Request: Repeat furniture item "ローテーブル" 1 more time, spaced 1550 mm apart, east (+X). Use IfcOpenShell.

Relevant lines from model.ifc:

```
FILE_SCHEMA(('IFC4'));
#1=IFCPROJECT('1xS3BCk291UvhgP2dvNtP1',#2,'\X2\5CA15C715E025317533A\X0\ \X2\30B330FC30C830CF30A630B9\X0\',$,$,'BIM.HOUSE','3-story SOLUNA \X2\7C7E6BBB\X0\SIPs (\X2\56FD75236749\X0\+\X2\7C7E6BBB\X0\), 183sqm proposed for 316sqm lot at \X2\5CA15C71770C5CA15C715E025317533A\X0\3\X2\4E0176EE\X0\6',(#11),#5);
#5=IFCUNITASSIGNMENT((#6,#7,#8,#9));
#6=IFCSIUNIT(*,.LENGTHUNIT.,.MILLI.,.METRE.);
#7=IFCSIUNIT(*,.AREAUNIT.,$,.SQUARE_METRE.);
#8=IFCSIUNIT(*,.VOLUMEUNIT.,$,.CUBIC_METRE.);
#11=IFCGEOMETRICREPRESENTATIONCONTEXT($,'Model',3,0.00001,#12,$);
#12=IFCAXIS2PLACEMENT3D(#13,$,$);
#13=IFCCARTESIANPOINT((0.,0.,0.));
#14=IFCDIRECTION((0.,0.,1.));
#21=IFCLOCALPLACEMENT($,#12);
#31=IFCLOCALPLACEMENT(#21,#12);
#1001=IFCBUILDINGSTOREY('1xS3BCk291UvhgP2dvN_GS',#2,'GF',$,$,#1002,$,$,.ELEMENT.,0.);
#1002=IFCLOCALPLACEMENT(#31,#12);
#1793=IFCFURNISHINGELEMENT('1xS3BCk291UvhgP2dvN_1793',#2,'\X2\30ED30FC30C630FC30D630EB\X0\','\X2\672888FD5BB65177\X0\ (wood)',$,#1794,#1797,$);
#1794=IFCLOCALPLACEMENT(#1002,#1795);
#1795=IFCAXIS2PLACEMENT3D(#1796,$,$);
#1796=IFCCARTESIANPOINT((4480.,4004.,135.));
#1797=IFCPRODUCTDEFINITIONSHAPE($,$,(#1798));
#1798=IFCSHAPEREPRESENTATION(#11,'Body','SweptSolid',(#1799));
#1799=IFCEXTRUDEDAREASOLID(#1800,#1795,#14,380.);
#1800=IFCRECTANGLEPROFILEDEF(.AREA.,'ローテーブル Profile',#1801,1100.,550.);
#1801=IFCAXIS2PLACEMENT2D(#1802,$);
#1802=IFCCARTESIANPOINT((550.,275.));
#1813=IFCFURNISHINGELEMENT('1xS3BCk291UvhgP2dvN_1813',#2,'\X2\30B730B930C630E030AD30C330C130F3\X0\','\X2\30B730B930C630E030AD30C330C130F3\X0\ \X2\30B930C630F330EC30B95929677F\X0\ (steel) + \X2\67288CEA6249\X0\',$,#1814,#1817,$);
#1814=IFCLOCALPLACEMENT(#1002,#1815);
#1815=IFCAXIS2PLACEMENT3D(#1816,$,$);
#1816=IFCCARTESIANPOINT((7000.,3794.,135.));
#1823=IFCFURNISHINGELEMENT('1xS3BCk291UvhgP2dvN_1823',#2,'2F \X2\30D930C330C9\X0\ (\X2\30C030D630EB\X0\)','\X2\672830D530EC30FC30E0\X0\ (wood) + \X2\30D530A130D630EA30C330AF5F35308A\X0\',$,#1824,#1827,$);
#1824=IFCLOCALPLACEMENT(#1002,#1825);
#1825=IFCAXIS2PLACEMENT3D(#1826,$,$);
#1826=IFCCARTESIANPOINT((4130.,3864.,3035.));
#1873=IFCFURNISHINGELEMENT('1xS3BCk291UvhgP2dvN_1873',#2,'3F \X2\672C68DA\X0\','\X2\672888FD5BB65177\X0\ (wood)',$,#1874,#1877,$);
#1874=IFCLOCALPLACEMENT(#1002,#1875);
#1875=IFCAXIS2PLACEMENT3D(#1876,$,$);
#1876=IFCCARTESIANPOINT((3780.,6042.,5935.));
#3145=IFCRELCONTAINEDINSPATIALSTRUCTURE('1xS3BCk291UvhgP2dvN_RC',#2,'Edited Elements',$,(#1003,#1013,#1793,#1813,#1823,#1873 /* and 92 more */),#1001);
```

```python
import numpy as np
import ifcopenshell
import ifcopenshell.api.geometry
import ifcopenshell.api.root
import ifcopenshell.util.element
import ifcopenshell.util.placement
import ifcopenshell.util.unit

model = ifcopenshell.open("model.ifc")
unit_scale = ifcopenshell.util.unit.calculate_unit_scale(model)


def reuse_history(source, copy):
    """copy_class also copies each property set's owner history, people and application; keep the originals."""
    for rel in copy.IsDefinedBy:
        if rel.is_a("IfcRelDefinesByProperties") and (history := rel.RelatingPropertyDefinition.OwnerHistory):
            rel.RelatingPropertyDefinition.OwnerHistory = source.OwnerHistory
            ifcopenshell.util.element.remove_deep2(model, history)


source = model.by_guid("1xS3BCk291UvhgP2dvN_1793")
base = ifcopenshell.util.placement.get_local_placement(source.ObjectPlacement)
step = np.array([1.0, 0.0, 0.0]) * 1.55 / unit_scale

for i in range(1, 2):
    copy = ifcopenshell.api.root.copy_class(model, product=source)
    copy.Representation = ifcopenshell.util.element.copy_deep(
        model, source.Representation, exclude=["IfcGeometricRepresentationContext", "IfcRepresentationMap"]
    )
    reuse_history(source, copy)
    matrix = base.copy()
    matrix[:3, 3] += i * step
    print("added at", matrix[:3, 3].round(3) + 0.0)
    ifcopenshell.api.geometry.edit_object_placement(model, product=copy, matrix=matrix, is_si=False)

model.write("model_v2.ifc")
```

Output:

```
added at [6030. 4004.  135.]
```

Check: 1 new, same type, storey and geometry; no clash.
